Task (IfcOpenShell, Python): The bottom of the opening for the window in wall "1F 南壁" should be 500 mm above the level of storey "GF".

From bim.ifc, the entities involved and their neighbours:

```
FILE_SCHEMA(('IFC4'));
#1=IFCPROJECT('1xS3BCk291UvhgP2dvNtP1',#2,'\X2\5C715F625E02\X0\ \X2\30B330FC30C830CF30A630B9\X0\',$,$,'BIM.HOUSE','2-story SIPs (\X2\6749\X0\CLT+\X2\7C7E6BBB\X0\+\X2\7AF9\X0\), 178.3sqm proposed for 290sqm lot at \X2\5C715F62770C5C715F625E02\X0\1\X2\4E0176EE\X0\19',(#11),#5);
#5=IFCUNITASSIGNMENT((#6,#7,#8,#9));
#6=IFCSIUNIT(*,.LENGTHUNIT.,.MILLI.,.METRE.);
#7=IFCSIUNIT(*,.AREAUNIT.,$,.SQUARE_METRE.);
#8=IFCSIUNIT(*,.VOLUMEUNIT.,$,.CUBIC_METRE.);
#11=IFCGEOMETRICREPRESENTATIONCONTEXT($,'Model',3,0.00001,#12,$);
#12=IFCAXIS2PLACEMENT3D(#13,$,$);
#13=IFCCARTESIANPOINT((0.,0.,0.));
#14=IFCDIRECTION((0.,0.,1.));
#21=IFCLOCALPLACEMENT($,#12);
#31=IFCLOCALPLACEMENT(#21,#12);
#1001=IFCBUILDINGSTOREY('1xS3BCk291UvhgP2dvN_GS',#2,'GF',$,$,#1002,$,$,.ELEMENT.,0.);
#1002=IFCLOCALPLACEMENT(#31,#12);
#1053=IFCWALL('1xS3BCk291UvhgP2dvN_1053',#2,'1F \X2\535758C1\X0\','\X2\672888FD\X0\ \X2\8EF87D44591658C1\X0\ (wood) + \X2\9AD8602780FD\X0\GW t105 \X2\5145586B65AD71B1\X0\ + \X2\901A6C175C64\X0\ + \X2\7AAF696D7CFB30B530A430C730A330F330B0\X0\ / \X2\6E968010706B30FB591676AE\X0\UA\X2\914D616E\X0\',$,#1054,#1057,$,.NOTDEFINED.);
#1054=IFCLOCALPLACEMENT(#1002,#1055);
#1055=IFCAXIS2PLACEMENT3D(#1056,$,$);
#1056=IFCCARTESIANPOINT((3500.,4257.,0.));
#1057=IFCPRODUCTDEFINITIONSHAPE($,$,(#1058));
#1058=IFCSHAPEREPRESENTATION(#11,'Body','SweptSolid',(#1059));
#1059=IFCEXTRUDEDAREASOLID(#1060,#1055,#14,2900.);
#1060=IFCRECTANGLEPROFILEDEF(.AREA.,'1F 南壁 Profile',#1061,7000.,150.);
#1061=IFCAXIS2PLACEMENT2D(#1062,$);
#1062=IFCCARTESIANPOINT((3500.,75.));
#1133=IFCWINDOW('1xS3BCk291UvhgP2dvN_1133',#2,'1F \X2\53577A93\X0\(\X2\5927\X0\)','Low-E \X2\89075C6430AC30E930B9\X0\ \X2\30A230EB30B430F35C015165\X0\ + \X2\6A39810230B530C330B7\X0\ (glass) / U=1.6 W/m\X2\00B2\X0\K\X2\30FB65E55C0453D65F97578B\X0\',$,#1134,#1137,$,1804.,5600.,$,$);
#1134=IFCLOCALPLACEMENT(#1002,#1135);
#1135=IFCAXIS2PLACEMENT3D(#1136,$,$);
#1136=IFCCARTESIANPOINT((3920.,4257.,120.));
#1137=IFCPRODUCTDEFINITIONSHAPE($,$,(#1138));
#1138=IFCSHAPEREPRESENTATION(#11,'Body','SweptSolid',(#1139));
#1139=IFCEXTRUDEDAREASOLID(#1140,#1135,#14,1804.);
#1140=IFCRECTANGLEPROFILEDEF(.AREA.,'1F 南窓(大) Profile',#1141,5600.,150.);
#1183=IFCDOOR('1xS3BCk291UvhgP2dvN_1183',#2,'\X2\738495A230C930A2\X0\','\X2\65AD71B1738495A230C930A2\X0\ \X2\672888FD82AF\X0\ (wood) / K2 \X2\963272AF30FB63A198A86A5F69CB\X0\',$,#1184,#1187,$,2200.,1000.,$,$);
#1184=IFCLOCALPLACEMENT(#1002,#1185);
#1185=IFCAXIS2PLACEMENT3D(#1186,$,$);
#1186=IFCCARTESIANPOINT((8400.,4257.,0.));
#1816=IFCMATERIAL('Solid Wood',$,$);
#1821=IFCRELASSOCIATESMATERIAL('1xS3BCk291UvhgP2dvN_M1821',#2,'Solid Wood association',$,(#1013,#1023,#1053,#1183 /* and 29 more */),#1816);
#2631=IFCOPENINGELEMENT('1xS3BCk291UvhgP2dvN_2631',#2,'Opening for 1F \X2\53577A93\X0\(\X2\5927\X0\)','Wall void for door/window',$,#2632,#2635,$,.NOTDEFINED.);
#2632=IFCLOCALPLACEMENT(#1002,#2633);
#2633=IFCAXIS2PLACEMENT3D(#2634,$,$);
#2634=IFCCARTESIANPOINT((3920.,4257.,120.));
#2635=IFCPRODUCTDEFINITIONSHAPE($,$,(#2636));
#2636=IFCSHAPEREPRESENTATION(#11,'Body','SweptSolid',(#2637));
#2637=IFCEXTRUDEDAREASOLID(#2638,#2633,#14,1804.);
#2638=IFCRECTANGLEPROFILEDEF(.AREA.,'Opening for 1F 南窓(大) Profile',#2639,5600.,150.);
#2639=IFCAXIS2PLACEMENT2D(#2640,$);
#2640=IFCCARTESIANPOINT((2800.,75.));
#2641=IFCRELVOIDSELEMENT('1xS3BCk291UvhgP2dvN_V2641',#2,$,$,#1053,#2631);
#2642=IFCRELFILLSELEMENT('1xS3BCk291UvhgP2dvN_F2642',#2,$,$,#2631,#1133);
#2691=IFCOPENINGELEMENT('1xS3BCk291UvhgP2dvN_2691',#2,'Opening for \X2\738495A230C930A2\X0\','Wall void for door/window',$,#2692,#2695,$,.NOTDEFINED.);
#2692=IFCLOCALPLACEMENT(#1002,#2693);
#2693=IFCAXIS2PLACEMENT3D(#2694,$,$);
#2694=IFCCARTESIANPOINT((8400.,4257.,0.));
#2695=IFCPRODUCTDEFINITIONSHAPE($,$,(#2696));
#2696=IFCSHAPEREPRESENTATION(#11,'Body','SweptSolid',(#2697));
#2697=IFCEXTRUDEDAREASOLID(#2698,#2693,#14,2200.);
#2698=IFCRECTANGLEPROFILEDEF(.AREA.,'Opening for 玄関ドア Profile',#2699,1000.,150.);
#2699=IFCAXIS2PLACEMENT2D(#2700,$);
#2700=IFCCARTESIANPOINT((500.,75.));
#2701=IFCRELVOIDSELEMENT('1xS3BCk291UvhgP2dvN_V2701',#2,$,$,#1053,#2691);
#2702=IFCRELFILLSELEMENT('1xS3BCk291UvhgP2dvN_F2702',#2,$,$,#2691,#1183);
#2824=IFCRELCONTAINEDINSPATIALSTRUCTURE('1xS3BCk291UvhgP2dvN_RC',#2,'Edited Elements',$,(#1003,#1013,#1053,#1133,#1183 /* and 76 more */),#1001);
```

```python
import numpy as np
import ifcopenshell
import ifcopenshell.api.geometry
import ifcopenshell.geom
import ifcopenshell.util.element
import ifcopenshell.util.placement
import ifcopenshell.util.shape
import ifcopenshell.util.unit

model = ifcopenshell.open("bim.ifc")
unit_scale = ifcopenshell.util.unit.calculate_unit_scale(model)

window = model.by_guid("1xS3BCk291UvhgP2dvN_1133")
opening = window.FillsVoids[0].RelatingOpeningElement
storey = ifcopenshell.util.element.get_container(window, ifc_class="IfcBuildingStorey")
level = ifcopenshell.util.placement.get_local_placement(storey.ObjectPlacement)[2, 3]

# The opening's origin need not be at the sill, so measure its lowest point.
shape = ifcopenshell.geom.create_shape(ifcopenshell.geom.settings(), opening)
bottom = ifcopenshell.util.shape.get_shape_bottom_elevation(shape, shape.geometry) / unit_scale
dz = level + 500.0 - bottom

shift = np.array([0.0, 0.0, dz])
# The window is not placed relative to its opening, so move both.
for product in (opening, window):
    matrix = ifcopenshell.util.placement.get_local_placement(product.ObjectPlacement)
    matrix[:3, 3] += shift
    ifcopenshell.api.geometry.edit_object_placement(model, product=product, matrix=matrix, is_si=False)

print(f"moved by {dz * unit_scale:+.3f} m")

model.write("bim_updated.ifc")
```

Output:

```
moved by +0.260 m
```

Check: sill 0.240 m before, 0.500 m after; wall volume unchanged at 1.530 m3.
